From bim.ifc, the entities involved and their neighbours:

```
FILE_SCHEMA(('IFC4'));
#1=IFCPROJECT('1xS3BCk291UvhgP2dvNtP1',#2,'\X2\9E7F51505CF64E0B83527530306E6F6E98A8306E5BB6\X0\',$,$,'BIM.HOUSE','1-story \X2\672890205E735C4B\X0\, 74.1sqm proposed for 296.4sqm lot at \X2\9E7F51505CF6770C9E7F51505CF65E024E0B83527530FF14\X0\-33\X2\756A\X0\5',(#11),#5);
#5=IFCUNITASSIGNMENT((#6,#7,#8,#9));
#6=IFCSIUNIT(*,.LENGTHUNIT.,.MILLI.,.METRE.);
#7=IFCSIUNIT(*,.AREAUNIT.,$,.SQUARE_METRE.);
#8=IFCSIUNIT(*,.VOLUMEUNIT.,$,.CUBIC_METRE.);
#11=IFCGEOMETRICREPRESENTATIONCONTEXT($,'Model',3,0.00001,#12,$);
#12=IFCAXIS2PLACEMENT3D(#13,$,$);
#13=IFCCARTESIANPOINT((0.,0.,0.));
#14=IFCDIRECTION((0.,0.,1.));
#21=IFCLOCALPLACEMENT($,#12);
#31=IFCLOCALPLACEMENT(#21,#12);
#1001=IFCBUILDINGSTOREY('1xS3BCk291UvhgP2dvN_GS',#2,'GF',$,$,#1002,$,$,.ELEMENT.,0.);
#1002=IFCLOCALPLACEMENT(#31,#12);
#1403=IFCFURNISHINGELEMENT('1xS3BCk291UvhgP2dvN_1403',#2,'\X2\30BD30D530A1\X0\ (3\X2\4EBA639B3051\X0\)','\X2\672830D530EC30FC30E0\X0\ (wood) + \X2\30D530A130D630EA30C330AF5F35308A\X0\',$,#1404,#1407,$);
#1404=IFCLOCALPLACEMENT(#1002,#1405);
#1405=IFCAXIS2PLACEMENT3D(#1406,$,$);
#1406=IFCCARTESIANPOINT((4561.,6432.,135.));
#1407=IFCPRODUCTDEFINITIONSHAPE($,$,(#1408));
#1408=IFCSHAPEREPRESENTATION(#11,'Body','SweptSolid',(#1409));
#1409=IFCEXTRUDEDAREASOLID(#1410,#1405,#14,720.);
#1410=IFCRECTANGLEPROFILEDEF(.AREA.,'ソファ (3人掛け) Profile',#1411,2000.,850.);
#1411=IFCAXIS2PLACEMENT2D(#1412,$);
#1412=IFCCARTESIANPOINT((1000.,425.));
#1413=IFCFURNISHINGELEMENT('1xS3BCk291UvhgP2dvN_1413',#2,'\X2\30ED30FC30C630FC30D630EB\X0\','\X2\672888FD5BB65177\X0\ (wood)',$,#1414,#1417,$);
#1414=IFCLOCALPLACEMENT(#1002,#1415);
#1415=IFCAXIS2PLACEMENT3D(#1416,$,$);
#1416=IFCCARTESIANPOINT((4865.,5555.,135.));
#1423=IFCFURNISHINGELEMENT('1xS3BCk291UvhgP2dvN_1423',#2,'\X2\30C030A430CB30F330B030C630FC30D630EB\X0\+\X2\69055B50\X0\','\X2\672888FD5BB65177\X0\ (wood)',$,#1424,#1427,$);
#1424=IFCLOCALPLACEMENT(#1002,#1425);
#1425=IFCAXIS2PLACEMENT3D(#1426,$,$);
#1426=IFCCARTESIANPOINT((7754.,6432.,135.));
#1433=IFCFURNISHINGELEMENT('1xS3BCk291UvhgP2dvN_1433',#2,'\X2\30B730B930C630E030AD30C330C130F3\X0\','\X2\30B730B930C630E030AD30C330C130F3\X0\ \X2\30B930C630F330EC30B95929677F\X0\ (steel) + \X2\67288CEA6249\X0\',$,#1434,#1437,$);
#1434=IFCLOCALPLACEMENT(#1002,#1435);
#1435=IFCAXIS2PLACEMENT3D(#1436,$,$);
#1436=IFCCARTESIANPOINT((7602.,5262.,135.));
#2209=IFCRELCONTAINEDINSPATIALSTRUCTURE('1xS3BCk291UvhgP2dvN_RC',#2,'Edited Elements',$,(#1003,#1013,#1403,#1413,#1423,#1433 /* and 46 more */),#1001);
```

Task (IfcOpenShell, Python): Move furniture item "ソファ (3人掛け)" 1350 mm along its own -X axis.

```python
import ifcopenshell
import ifcopenshell.api.geometry
import ifcopenshell.util.placement

model = ifcopenshell.open("bim.ifc")

item = model.by_guid("1xS3BCk291UvhgP2dvN_1403")
matrix = ifcopenshell.util.placement.get_local_placement(item.ObjectPlacement)
matrix[:3, 3] -= matrix[:3, 0] * 1350.0
ifcopenshell.api.geometry.edit_object_placement(model, product=item, matrix=matrix, is_si=False)

print(ifcopenshell.util.placement.get_local_placement(item.ObjectPlacement).round(3) + 0.0)

model.write("bim_edited.ifc")
```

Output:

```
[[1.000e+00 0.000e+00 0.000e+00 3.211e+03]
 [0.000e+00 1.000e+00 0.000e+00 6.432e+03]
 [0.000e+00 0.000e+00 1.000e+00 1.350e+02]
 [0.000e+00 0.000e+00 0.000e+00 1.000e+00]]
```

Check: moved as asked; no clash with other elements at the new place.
